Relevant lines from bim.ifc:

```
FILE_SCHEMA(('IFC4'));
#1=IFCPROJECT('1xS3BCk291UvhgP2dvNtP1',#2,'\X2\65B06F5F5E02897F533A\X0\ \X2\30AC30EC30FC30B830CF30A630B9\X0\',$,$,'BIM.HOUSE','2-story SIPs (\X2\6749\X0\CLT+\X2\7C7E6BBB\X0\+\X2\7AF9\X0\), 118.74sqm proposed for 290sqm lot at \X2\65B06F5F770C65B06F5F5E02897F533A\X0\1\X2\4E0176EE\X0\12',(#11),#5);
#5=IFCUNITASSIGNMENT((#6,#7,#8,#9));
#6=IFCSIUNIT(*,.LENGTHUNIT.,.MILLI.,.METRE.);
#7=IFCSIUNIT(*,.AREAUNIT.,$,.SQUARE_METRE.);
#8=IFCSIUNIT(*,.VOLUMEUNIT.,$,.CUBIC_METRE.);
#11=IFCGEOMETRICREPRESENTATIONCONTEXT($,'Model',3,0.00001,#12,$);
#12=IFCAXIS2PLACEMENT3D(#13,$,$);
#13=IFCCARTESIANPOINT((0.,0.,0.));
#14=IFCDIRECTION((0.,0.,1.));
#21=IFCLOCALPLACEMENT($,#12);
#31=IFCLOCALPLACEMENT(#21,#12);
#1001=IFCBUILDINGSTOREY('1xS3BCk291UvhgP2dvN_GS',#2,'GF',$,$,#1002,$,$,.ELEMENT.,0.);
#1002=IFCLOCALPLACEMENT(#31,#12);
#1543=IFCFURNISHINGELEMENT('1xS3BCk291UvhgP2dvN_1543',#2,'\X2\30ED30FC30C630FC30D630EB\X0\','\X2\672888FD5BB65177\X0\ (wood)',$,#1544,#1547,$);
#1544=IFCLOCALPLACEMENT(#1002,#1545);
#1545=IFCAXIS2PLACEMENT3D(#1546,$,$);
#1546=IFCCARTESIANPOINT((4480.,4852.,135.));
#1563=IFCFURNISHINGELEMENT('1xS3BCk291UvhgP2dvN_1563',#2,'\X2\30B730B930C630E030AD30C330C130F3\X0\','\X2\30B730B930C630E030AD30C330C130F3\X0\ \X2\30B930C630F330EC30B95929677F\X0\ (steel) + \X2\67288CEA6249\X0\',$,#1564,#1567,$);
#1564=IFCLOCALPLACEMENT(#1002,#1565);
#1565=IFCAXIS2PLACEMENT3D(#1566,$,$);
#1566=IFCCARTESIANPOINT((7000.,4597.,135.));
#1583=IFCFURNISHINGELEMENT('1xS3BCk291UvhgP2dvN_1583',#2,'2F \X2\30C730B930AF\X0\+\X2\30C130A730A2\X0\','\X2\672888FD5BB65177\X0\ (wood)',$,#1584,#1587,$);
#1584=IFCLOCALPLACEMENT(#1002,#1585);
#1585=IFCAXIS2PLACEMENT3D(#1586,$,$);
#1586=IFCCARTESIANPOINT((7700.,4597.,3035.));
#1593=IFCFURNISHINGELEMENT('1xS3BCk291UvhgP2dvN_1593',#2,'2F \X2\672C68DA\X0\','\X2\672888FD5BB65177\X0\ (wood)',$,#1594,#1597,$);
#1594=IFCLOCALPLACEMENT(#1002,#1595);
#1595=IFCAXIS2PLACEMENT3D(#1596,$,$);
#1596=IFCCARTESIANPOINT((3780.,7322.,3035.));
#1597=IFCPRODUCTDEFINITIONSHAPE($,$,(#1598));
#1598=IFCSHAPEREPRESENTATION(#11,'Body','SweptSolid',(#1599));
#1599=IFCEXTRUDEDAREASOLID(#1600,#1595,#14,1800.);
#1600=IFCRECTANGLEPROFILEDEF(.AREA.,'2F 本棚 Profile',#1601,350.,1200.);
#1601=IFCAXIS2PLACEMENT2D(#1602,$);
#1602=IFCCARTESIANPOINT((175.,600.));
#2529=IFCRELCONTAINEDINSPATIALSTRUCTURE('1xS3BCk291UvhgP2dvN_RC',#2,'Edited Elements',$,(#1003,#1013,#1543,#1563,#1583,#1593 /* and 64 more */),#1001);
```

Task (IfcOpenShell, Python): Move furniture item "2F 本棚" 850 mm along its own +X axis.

```python
import ifcopenshell
import ifcopenshell.api.geometry
import ifcopenshell.util.placement

model = ifcopenshell.open("bim.ifc")

item = model.by_guid("1xS3BCk291UvhgP2dvN_1593")
matrix = ifcopenshell.util.placement.get_local_placement(item.ObjectPlacement)
matrix[:3, 3] += matrix[:3, 0] * 850.0
ifcopenshell.api.geometry.edit_object_placement(model, product=item, matrix=matrix, is_si=False)

print(ifcopenshell.util.placement.get_local_placement(item.ObjectPlacement).round(3) + 0.0)

model.write("bim-out.ifc")
```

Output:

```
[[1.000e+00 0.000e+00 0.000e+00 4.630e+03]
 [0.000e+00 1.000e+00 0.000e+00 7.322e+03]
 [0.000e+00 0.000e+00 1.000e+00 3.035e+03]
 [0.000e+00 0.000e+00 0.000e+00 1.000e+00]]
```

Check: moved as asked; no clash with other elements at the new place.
